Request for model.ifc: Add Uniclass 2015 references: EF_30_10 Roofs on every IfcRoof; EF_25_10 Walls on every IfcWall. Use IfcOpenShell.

First a look at what the model holds.

```python
import ifcopenshell

model = ifcopenshell.open("model.ifc")
print(model.schema)
print("classifications:", [c.Name for c in model.by_type("IfcClassification")])
for ifc_class in ("IfcDoor", "IfcRoof", "IfcStair", "IfcWall", "IfcWindow"):
    print(ifc_class, len(model.by_type(ifc_class)))
```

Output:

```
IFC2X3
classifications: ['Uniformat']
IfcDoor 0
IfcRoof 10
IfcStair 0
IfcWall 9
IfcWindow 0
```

```python
import ifcopenshell
import ifcopenshell.api.classification

model = ifcopenshell.open("model.ifc")

# IFC2X3 requires Source and Edition and has no link from the project to the system.
system = model.create_entity("IfcClassification", Source="NBS", Edition="2015", Name="Uniclass 2015")

codes = {
    "IfcRoof": ("EF_30_10", "Roofs"),
    "IfcWall": ("EF_25_10", "Walls"),
}
for ifc_class, (code, name) in codes.items():
    products = model.by_type(ifc_class)
    ifcopenshell.api.classification.add_reference(
        model, products=products, classification=system, identification=code, name=name
    )
    print(code, len(products))

model.write("model_v2.ifc")
```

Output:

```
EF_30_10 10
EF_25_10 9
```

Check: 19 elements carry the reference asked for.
